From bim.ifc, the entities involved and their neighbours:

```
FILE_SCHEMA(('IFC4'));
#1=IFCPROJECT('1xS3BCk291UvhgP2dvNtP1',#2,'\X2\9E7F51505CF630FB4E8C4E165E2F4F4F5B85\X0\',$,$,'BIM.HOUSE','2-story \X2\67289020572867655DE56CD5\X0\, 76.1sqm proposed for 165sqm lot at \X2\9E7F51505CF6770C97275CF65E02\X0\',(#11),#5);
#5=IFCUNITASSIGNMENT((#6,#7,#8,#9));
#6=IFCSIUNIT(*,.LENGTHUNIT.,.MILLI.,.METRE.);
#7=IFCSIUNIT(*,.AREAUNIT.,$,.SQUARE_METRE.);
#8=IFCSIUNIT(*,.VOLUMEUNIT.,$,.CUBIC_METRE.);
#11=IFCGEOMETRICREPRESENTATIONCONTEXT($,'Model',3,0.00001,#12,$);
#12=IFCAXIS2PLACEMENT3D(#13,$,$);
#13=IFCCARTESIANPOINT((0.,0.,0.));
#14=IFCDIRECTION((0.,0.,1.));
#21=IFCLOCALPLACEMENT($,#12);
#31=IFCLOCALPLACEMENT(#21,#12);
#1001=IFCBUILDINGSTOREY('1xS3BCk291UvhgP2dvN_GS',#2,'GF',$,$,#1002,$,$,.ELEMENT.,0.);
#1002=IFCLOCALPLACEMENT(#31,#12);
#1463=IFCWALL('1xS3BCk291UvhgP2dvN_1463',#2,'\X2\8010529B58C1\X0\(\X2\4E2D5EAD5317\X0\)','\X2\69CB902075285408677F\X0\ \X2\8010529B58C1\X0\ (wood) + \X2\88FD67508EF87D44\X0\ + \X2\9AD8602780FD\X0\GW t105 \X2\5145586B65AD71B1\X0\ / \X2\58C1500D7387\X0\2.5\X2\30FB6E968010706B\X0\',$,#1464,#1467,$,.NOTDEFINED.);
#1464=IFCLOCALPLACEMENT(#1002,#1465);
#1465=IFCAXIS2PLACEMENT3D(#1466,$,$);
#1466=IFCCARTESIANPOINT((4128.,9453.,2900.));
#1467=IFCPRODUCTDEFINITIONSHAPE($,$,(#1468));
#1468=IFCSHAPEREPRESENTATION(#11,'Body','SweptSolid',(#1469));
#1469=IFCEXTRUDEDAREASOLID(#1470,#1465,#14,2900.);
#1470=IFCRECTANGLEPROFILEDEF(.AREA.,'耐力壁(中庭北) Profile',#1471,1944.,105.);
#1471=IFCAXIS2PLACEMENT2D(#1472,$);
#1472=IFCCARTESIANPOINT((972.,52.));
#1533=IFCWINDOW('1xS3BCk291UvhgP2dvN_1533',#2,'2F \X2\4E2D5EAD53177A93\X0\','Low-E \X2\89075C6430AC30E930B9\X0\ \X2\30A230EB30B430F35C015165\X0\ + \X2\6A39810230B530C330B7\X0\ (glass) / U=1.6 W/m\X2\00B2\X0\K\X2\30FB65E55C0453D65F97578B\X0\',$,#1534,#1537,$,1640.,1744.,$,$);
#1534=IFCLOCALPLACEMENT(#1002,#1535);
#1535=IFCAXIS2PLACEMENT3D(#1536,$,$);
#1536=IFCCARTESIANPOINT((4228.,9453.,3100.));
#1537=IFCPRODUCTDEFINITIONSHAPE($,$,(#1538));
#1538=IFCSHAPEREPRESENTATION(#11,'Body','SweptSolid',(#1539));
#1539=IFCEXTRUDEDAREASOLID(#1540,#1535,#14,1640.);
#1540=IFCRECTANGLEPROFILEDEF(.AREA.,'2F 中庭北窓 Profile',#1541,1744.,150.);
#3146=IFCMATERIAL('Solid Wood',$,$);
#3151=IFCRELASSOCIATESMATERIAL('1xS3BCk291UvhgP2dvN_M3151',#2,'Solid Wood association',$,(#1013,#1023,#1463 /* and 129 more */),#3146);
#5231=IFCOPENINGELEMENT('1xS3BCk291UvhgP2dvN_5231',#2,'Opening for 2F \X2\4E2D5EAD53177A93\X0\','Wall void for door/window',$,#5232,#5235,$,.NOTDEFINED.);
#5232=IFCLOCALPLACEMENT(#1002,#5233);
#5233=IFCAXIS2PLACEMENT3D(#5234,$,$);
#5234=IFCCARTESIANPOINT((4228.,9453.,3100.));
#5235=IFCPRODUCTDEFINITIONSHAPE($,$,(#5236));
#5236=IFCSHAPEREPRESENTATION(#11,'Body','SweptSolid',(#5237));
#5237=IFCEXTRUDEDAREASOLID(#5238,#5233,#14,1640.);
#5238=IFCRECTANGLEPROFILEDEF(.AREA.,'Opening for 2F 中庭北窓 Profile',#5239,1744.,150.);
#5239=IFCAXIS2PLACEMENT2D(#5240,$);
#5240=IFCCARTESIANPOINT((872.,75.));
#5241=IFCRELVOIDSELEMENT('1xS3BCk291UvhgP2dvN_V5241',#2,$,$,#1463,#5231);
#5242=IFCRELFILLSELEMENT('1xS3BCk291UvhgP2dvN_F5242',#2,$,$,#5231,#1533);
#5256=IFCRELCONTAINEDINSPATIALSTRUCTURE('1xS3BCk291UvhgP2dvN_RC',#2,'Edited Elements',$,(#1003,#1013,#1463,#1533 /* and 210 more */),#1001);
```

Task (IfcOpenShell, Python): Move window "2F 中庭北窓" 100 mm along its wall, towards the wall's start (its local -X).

```python
import ifcopenshell
import ifcopenshell.api.geometry
import ifcopenshell.util.placement

model = ifcopenshell.open("bim.ifc")

window = model.by_id(1533)
opening = window.FillsVoids[0].RelatingOpeningElement
wall = opening.VoidsElements[0].RelatingBuildingElement

wall_matrix = ifcopenshell.util.placement.get_local_placement(wall.ObjectPlacement)
shift = wall_matrix[:3, 0] * -100.0
before = ifcopenshell.util.placement.get_local_placement(window.ObjectPlacement)[:3, 3].copy()

# The window is not placed relative to its opening, so move both.
for product in (opening, window):
    matrix = ifcopenshell.util.placement.get_local_placement(product.ObjectPlacement)
    matrix[:3, 3] += shift
    ifcopenshell.api.geometry.edit_object_placement(model, product=product, matrix=matrix, is_si=False)

after = ifcopenshell.util.placement.get_local_placement(window.ObjectPlacement)[:3, 3]
print("window moved by", (after - before).round(3) + 0.0)

model.write("bim_rev.ifc")
```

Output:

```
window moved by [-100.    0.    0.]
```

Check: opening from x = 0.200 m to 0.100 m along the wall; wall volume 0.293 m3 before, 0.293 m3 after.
